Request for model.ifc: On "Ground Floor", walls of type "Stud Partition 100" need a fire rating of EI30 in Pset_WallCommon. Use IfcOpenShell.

First a look at what the model holds.

```python
import ifcopenshell
import ifcopenshell.util.element

model = ifcopenshell.open("model.ifc")
print(model.schema)
storey = next(s for s in model.by_type("IfcBuildingStorey") if s.Name == "Ground Floor")
walls = [e for e in ifcopenshell.util.element.get_decomposition(storey) if e.is_a("IfcWall")]
seen = {}
for e in walls:
    element_type = ifcopenshell.util.element.get_type(e)
    key = (element_type.Name if element_type != e and element_type else None, ifcopenshell.util.element.get_pset(e, "Pset_WallCommon", "FireRating"))
    seen[key] = seen.get(key, 0) + 1
for (name, value), count in sorted(seen.items(), key=str):
    print(count, "x", name, "|", value)
```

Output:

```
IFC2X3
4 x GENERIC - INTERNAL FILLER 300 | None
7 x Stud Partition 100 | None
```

```python
import ifcopenshell
import ifcopenshell.api.pset
import ifcopenshell.util.element

model = ifcopenshell.open("model.ifc")

storey = next(s for s in model.by_type("IfcBuildingStorey") if s.Name == "Ground Floor")
walls = [e for e in ifcopenshell.util.element.get_decomposition(storey) if e.is_a("IfcWall")]

count = 0
for e in walls:
    element_type = ifcopenshell.util.element.get_type(e)
    if element_type in (None, e) or element_type.Name != "Stud Partition 100":
        continue
    # add_pset returns the element's existing set when there is one.
    pset = ifcopenshell.api.pset.add_pset(model, product=e, name="Pset_WallCommon")
    ifcopenshell.api.pset.edit_pset(model, pset=pset, properties={"FireRating": "EI30"})
    count += 1

print(count, "walls updated")

model.write("model_updated.ifc")
```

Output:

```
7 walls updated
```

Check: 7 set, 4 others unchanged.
